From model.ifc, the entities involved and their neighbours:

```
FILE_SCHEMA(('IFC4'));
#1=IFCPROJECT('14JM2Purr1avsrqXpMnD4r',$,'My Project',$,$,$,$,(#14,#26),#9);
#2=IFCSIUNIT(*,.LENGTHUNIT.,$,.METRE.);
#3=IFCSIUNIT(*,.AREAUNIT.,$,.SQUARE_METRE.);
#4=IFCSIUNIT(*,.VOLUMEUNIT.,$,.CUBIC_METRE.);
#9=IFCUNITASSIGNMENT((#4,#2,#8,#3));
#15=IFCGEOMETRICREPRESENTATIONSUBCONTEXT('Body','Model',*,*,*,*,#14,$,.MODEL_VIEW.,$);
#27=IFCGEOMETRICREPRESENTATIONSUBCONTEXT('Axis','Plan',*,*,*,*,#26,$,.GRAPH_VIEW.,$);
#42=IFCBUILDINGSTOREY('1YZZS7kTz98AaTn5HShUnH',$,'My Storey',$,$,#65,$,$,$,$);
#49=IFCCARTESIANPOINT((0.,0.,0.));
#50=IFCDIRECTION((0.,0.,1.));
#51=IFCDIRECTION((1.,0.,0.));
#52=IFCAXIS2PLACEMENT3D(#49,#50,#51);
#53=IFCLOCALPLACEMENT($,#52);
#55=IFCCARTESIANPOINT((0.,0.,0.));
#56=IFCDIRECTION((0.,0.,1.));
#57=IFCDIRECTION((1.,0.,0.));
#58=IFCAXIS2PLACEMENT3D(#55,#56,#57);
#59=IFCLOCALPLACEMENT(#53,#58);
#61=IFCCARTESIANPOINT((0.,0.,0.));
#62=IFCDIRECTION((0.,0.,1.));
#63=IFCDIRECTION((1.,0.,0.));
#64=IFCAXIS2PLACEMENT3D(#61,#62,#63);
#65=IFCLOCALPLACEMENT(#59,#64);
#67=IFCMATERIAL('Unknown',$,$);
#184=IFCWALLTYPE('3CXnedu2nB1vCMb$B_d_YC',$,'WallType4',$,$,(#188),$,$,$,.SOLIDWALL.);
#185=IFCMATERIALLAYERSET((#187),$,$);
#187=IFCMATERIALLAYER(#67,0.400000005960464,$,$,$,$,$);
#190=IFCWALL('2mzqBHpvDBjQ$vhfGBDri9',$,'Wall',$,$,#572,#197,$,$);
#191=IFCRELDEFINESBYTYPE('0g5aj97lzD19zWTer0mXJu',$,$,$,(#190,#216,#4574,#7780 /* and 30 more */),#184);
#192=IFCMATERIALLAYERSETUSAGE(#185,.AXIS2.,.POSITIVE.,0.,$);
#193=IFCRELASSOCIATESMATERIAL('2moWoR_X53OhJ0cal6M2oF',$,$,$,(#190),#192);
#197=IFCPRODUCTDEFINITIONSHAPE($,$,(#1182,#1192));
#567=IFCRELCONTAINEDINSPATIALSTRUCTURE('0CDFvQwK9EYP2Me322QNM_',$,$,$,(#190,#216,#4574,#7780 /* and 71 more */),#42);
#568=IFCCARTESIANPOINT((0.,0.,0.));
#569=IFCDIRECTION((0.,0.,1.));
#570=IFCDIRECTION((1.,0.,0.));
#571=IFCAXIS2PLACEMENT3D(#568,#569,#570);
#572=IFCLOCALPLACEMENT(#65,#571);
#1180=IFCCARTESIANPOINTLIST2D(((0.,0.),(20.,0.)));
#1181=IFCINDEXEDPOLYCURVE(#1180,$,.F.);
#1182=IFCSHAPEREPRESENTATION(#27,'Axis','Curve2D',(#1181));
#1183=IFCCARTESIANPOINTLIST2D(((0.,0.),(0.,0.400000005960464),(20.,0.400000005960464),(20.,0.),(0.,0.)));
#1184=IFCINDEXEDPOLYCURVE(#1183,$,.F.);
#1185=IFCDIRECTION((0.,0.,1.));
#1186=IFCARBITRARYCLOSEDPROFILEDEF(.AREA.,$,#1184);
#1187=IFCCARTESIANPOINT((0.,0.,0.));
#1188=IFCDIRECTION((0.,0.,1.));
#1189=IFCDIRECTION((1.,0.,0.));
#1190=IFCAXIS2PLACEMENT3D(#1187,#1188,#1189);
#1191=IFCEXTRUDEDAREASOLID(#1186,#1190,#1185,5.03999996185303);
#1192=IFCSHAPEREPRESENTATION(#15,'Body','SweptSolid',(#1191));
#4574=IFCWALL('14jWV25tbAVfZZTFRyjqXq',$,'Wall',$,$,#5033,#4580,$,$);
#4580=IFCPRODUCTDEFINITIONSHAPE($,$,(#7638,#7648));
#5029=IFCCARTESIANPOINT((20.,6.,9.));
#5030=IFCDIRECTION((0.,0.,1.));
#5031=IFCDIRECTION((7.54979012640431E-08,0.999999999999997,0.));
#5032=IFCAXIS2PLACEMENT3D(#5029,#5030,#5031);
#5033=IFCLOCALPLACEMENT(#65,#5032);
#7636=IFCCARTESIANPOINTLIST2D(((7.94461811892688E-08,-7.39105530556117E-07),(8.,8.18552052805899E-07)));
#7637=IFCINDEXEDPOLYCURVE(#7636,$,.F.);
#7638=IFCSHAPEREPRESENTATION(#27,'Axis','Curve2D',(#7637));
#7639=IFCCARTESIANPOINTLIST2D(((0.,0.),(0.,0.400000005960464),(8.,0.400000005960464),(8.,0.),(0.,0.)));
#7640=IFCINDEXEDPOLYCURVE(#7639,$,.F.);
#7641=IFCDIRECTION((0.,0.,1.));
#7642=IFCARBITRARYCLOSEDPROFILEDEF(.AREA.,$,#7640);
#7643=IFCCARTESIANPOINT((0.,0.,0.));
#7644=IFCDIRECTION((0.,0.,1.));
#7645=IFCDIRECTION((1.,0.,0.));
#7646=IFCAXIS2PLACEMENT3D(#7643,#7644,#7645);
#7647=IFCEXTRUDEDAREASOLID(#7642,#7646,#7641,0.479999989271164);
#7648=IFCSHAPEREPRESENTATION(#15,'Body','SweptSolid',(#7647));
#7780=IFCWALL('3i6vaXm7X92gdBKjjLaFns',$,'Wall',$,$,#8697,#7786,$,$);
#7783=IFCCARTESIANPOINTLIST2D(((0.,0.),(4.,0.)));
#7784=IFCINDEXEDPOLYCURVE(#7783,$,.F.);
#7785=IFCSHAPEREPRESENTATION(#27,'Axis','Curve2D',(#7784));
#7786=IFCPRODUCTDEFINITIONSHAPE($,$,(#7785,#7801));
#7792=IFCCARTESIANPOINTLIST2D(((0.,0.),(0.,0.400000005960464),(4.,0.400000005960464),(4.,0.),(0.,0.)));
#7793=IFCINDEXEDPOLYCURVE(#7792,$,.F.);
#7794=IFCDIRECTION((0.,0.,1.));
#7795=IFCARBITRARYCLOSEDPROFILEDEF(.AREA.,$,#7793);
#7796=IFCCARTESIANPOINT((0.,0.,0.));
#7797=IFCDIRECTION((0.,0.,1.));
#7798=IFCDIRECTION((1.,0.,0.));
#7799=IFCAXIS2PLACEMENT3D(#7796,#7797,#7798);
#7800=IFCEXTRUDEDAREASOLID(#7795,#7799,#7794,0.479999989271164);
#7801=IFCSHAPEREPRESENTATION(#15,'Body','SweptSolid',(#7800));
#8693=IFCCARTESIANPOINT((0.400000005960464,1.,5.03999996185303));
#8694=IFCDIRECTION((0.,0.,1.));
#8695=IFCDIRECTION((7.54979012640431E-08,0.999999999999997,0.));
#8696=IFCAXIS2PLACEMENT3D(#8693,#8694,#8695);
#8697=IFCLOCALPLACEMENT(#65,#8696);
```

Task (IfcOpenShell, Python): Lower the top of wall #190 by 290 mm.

```python
import ifcopenshell
import ifcopenshell.geom
import ifcopenshell.util.representation
import ifcopenshell.util.shape
import ifcopenshell.util.unit

model = ifcopenshell.open("model.ifc")
unit_scale = ifcopenshell.util.unit.calculate_unit_scale(model)
settings = ifcopenshell.geom.settings()


def volume(element):
    """Net volume in cubic metres, openings subtracted."""
    shape = ifcopenshell.geom.create_shape(settings, element)
    return ifcopenshell.util.shape.get_volume(shape.geometry)


wall = model.by_guid("2mzqBHpvDBjQ$vhfGBDri9")
before = volume(wall)

body = ifcopenshell.util.representation.get_representation(wall, "Model", "Body")
solid = body.Items[0]
old_height = solid.Depth
solid.Depth -= 0.29 / unit_scale
after = volume(wall)

print(f"height {old_height:g} -> {solid.Depth:g}, volume {before:.3f} -> {after:.3f} m3")

model.write("model-out.ifc")
```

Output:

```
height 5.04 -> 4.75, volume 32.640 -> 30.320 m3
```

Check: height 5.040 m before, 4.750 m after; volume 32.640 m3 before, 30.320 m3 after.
